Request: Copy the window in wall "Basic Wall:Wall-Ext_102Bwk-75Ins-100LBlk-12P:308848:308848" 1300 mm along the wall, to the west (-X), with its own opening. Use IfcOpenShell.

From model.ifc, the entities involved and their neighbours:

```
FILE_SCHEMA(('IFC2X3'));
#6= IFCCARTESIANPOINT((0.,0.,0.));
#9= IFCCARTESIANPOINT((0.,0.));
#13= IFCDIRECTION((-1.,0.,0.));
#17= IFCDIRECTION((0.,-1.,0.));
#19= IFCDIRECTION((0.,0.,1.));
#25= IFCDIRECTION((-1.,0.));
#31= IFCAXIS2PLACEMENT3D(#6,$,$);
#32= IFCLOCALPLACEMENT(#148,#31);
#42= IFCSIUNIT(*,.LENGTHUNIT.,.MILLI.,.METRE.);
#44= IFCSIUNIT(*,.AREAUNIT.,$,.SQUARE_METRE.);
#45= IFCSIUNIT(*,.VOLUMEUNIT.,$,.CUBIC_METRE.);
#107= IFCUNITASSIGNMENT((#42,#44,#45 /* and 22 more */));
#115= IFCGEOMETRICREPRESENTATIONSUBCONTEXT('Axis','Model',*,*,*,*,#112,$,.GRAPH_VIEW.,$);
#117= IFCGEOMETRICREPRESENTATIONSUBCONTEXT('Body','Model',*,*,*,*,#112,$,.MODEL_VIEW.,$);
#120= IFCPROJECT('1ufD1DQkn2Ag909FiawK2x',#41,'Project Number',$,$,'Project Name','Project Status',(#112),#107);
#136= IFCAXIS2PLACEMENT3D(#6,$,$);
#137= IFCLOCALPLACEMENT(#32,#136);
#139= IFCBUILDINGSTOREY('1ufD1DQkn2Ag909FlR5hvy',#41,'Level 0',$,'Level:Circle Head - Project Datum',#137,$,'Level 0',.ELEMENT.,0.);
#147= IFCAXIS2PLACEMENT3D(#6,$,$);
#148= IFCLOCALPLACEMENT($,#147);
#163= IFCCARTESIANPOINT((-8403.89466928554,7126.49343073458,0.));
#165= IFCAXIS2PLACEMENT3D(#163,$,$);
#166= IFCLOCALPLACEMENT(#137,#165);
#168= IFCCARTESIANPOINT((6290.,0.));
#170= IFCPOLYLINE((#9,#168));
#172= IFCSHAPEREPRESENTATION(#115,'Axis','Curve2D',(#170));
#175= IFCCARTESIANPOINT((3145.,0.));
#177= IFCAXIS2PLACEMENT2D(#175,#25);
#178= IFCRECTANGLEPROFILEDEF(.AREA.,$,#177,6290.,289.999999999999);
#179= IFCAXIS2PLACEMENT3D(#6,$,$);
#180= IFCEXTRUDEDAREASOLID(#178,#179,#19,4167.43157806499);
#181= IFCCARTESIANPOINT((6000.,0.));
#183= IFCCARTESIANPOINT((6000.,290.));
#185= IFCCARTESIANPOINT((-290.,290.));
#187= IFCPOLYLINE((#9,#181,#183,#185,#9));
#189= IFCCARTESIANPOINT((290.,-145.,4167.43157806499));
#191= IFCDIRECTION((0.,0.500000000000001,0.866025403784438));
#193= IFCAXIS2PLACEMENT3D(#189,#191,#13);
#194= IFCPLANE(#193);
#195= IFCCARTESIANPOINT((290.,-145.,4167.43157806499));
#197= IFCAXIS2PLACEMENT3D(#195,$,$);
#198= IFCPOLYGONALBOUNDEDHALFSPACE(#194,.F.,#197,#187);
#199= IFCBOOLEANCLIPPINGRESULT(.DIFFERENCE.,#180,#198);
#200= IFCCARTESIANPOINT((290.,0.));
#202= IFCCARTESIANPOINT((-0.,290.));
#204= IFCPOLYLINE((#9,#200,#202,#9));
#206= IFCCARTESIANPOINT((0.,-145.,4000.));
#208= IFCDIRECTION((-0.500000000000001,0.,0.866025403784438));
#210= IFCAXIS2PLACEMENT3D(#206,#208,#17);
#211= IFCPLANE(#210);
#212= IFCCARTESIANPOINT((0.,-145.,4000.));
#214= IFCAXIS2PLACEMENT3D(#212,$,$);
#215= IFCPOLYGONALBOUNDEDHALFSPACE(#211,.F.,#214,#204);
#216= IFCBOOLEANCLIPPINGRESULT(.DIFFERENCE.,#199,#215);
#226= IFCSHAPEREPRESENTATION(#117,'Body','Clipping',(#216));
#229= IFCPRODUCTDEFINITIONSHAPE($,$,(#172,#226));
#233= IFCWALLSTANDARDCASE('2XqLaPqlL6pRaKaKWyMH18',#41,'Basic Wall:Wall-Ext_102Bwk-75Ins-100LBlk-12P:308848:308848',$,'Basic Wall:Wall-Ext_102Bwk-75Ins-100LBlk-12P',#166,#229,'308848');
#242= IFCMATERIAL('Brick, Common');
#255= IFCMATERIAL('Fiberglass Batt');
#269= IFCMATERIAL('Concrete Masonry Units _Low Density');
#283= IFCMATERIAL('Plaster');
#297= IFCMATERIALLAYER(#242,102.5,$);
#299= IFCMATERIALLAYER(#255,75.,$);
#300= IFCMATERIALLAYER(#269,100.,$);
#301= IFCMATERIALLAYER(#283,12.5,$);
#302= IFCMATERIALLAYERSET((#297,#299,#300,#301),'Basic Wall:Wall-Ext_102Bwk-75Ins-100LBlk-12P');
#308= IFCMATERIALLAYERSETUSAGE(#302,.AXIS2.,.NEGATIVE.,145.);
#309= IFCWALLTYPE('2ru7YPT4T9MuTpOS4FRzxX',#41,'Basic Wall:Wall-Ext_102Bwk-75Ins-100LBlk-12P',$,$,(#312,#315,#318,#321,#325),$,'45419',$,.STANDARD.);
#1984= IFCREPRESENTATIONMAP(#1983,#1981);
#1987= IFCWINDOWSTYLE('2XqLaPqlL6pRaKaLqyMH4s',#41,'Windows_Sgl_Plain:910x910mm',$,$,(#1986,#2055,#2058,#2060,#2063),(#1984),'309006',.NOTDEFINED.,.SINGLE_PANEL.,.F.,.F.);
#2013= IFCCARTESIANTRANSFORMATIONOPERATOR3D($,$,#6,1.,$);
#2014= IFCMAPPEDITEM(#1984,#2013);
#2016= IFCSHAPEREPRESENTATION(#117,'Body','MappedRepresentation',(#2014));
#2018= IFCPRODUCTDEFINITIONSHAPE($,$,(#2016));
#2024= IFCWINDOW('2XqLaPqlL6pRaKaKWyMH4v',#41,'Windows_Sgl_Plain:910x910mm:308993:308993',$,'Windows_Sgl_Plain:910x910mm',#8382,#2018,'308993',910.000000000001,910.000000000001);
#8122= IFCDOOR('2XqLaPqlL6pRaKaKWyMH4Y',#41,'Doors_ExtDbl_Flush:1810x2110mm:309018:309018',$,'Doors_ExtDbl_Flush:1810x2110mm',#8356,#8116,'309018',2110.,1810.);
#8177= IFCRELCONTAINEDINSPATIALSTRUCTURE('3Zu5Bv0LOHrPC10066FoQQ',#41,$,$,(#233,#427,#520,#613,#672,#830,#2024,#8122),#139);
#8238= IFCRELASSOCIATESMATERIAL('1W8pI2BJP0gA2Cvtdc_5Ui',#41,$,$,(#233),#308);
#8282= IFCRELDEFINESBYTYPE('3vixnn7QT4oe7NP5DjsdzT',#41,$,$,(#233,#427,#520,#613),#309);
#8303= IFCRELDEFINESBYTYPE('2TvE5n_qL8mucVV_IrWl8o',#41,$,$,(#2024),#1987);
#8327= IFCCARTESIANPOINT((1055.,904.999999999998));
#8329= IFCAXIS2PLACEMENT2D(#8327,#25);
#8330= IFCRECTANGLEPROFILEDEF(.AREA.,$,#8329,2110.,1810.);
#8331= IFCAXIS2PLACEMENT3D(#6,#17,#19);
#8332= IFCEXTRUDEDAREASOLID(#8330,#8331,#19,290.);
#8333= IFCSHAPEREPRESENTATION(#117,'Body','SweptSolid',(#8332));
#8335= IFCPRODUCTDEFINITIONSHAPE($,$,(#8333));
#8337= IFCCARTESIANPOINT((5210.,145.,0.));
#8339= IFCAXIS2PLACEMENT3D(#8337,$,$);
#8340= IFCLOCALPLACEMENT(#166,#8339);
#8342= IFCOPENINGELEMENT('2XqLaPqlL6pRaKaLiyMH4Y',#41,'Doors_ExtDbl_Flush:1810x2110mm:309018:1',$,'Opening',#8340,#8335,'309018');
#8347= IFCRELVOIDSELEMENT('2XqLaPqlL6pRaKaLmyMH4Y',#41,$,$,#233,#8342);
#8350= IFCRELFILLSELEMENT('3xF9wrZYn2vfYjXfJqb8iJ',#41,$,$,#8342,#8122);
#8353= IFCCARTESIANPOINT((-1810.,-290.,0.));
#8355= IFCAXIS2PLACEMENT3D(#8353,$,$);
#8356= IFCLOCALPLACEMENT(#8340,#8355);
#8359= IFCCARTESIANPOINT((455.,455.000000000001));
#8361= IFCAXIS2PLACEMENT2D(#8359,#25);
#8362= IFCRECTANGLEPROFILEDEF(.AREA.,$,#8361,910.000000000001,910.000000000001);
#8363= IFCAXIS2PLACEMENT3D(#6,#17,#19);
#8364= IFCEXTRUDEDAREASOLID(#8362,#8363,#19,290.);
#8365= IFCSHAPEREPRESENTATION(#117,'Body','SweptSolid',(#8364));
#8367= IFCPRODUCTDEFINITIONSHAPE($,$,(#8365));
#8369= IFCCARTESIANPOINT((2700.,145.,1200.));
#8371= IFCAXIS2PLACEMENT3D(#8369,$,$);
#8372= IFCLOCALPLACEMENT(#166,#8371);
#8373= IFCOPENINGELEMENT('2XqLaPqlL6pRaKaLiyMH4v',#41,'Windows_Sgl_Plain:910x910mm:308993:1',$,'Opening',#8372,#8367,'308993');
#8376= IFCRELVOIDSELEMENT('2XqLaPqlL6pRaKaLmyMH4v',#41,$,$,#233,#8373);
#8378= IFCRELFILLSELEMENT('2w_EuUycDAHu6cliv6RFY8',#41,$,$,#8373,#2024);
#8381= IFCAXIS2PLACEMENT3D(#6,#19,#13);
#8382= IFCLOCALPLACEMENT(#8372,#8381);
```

```python
import ifcopenshell
import ifcopenshell.api.feature
import ifcopenshell.api.geometry
import ifcopenshell.api.root
import ifcopenshell.geom
import ifcopenshell.util.element
import ifcopenshell.util.placement
import ifcopenshell.util.shape

model = ifcopenshell.open("model.ifc")
settings = ifcopenshell.geom.settings()


def volume(element):
    """Net volume in cubic metres, openings subtracted."""
    shape = ifcopenshell.geom.create_shape(settings, element)
    return ifcopenshell.util.shape.get_volume(shape.geometry)


def reuse_history(source, copy):
    """copy_class also copies each property set's owner history, people and application; keep the originals."""
    for rel in copy.IsDefinedBy:
        if rel.is_a("IfcRelDefinesByProperties") and (history := rel.RelatingPropertyDefinition.OwnerHistory):
            rel.RelatingPropertyDefinition.OwnerHistory = source.OwnerHistory
            ifcopenshell.util.element.remove_deep2(model, history)


window = model.by_guid("2XqLaPqlL6pRaKaKWyMH4v")
opening = window.FillsVoids[0].RelatingOpeningElement
wall = opening.VoidsElements[0].RelatingBuildingElement
before = volume(wall)
shift = ifcopenshell.util.placement.get_local_placement(wall.ObjectPlacement)[:3, 0] * -1300.0

# copy_class copies the void relationship, type, container and properties, but no geometry.
new_opening = ifcopenshell.api.root.copy_class(model, product=opening)
new_opening.Representation = ifcopenshell.util.element.copy_deep(
    model, opening.Representation, exclude=["IfcGeometricRepresentationContext", "IfcRepresentationMap"]
)
new_opening.Name = "Windows_Sgl_Plain:910x910mm"
new_opening.Tag = None
new_window = ifcopenshell.api.root.copy_class(model, product=window)
new_window.Representation = ifcopenshell.util.element.copy_deep(
    model, window.Representation, exclude=["IfcGeometricRepresentationContext", "IfcRepresentationMap"]
)
new_window.Name = "Windows_Sgl_Plain:910x910mm"
new_window.Tag = None
reuse_history(window, new_window)
fills = ifcopenshell.api.feature.add_filling(model, opening=new_opening, element=new_window)
fills.OwnerHistory = new_window.OwnerHistory  # required in IFC2X3

for old, new in ((opening, new_opening), (window, new_window)):
    matrix = ifcopenshell.util.placement.get_local_placement(old.ObjectPlacement)
    matrix[:3, 3] += shift
    ifcopenshell.api.geometry.edit_object_placement(model, product=new, matrix=matrix, is_si=False)

after = volume(wall)

print(f"wall volume {before:.3f} -> {after:.3f} m3")

model.write("model_updated.ifc")
```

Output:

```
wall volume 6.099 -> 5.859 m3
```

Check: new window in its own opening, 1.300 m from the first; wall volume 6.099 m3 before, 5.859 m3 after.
